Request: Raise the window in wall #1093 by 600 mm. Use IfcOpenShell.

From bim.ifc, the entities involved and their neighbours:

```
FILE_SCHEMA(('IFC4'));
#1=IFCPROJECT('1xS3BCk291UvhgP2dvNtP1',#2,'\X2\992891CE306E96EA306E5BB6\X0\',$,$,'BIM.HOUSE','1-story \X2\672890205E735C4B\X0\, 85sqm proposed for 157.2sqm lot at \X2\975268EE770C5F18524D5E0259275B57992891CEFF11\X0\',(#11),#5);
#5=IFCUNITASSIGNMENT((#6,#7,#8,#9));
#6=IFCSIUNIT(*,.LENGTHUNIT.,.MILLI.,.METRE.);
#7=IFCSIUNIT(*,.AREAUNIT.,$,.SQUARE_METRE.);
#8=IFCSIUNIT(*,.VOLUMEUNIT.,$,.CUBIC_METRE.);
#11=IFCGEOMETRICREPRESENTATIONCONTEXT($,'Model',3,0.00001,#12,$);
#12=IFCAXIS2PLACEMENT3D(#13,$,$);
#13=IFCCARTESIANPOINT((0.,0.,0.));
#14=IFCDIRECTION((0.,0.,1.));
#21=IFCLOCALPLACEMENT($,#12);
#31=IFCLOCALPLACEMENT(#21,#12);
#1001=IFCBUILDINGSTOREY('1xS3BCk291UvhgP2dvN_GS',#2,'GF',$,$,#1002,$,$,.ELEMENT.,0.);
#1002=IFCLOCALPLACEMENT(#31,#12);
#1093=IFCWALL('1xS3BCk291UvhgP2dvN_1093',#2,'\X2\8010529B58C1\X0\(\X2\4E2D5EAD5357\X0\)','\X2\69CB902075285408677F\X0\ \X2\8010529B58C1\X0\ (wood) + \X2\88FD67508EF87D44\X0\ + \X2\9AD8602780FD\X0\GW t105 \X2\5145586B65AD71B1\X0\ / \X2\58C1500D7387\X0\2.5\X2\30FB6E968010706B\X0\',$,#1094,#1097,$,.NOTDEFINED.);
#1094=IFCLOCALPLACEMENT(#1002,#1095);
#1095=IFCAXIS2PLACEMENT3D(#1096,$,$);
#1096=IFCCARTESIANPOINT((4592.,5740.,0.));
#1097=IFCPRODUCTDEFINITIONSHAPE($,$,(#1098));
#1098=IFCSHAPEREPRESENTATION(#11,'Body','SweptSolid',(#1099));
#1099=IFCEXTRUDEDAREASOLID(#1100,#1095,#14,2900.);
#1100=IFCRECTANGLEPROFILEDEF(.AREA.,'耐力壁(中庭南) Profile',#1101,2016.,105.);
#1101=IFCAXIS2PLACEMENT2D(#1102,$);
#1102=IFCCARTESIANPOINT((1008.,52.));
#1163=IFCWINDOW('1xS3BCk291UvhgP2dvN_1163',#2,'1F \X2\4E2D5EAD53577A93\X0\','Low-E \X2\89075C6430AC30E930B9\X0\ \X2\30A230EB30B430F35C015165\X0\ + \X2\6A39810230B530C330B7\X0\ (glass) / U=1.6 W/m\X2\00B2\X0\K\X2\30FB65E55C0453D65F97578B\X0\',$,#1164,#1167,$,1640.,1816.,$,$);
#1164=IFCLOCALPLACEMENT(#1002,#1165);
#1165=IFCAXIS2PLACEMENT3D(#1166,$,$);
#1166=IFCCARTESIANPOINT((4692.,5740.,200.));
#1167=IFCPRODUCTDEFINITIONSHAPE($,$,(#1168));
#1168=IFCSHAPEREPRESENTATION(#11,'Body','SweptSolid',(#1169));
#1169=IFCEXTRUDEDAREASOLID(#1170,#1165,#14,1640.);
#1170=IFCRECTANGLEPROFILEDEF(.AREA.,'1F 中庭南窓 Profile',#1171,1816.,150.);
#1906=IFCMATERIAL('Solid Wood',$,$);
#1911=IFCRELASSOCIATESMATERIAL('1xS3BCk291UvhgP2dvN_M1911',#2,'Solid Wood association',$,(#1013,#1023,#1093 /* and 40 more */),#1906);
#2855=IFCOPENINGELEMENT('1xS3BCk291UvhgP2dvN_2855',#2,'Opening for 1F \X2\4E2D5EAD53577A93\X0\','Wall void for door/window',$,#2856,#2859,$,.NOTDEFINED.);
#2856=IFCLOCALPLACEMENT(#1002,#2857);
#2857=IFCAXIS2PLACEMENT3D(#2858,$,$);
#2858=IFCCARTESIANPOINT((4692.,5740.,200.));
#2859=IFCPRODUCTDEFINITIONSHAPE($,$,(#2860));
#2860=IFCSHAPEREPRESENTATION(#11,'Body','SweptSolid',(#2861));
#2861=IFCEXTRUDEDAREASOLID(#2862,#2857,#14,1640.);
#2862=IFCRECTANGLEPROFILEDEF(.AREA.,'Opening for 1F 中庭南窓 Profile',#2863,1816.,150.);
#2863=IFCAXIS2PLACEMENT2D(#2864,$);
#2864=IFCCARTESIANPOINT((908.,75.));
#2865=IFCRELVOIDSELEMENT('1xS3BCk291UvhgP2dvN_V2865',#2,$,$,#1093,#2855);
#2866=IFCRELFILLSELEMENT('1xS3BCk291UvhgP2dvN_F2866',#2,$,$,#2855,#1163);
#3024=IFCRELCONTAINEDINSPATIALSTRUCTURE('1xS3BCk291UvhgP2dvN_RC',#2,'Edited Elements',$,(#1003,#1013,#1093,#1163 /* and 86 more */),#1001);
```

```python
import numpy as np
import ifcopenshell
import ifcopenshell.api.geometry
import ifcopenshell.util.placement
import ifcopenshell.util.unit

model = ifcopenshell.open("bim.ifc")
unit_scale = ifcopenshell.util.unit.calculate_unit_scale(model)

window = model.by_guid("1xS3BCk291UvhgP2dvN_1163")
opening = window.FillsVoids[0].RelatingOpeningElement
dz = 0.6 / unit_scale

shift = np.array([0.0, 0.0, dz])
# The window is not placed relative to its opening, so move both.
for product in (opening, window):
    matrix = ifcopenshell.util.placement.get_local_placement(product.ObjectPlacement)
    matrix[:3, 3] += shift
    ifcopenshell.api.geometry.edit_object_placement(model, product=product, matrix=matrix, is_si=False)

print(f"moved by {dz * unit_scale:+.3f} m")

model.write("bim_edited.ifc")
```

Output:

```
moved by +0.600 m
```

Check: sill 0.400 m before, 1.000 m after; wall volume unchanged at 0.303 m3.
